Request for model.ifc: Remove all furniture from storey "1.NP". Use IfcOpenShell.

First a look at what the model holds.

```python
import ifcopenshell
import ifcopenshell.util.element

model = ifcopenshell.open("model.ifc")
print(model.schema)
storey = next(s for s in model.by_type("IfcBuildingStorey") if s.Name == "1.NP")
furniture = [e for e in ifcopenshell.util.element.get_decomposition(storey) if e.is_a("IfcFurnishingElement")]
seen = {}
for e in furniture:
    element_type = ifcopenshell.util.element.get_type(e)
    name = element_type.Name if element_type not in (None, e) else None
    seen[name] = seen.get(name, 0) + 1
for name, count in sorted(seen.items(), key=str):
    print(count, "x", name)
```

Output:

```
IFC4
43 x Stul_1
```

```python
import ifcopenshell
import ifcopenshell.api.root
import ifcopenshell.util.element

model = ifcopenshell.open("model.ifc")

storey = next(s for s in model.by_type("IfcBuildingStorey") if s.Name == "1.NP")
furniture = [e for e in ifcopenshell.util.element.get_decomposition(storey) if e.is_a("IfcFurnishingElement")]

for e in furniture:
    ifcopenshell.api.root.remove_product(model, product=e)
print(len(furniture), "removed")

model.write("model-out.ifc")
```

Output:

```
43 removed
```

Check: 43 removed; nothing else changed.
